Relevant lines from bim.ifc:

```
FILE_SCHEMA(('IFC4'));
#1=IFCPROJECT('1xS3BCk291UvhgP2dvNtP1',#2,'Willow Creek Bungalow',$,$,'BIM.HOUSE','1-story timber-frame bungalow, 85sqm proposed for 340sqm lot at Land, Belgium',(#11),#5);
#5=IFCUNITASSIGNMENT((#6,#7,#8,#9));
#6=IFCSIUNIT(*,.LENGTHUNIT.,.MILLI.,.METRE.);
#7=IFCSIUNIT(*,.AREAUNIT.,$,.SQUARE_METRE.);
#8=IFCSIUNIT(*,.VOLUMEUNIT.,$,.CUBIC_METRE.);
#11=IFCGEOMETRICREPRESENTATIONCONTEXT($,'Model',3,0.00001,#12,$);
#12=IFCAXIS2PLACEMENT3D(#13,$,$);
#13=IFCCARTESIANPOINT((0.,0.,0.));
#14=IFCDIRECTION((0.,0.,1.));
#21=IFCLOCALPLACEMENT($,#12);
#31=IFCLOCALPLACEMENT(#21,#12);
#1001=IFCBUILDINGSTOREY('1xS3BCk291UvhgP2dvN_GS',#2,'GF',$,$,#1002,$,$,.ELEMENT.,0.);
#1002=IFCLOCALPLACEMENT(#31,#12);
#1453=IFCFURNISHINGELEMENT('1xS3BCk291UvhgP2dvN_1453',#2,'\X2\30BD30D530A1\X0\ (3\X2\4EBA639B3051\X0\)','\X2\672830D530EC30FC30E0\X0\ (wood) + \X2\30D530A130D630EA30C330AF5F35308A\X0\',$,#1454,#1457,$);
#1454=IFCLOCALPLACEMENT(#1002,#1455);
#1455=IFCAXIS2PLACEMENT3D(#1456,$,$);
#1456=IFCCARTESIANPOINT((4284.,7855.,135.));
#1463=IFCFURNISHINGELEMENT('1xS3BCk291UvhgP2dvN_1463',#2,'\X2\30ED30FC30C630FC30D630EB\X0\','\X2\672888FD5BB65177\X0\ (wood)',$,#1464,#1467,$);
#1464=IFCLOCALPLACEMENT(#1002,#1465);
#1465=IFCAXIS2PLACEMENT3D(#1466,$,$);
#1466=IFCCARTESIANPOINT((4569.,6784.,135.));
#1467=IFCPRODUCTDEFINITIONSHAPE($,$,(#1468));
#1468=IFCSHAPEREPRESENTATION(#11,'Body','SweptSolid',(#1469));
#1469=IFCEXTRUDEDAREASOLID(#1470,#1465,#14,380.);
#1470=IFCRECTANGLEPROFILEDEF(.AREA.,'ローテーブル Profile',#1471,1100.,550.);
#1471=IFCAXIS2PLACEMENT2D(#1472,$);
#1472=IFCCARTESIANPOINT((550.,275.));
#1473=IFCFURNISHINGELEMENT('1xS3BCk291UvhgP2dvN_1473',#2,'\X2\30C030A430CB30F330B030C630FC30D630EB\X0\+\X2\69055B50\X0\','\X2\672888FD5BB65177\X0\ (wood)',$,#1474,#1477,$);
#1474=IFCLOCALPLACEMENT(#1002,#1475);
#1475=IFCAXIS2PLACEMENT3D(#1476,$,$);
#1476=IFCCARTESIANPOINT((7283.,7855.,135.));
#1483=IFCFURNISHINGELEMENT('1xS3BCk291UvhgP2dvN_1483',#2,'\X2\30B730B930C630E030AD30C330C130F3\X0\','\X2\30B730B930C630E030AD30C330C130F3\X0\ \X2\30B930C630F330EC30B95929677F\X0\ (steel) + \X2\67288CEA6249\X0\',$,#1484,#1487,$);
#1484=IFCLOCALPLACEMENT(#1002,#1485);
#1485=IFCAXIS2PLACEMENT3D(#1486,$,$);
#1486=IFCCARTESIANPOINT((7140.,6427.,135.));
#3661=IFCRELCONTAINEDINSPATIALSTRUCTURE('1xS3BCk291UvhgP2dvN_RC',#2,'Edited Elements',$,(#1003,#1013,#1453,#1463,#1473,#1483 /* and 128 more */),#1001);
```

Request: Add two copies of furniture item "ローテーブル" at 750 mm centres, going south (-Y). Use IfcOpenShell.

```python
import numpy as np
import ifcopenshell
import ifcopenshell.api.geometry
import ifcopenshell.api.root
import ifcopenshell.util.element
import ifcopenshell.util.placement
import ifcopenshell.util.unit

model = ifcopenshell.open("bim.ifc")
unit_scale = ifcopenshell.util.unit.calculate_unit_scale(model)


def reuse_history(source, copy):
    """copy_class also copies each property set's owner history, people and application; keep the originals."""
    for rel in copy.IsDefinedBy:
        if rel.is_a("IfcRelDefinesByProperties") and (history := rel.RelatingPropertyDefinition.OwnerHistory):
            rel.RelatingPropertyDefinition.OwnerHistory = source.OwnerHistory
            ifcopenshell.util.element.remove_deep2(model, history)


source = model.by_guid("1xS3BCk291UvhgP2dvN_1463")
base = ifcopenshell.util.placement.get_local_placement(source.ObjectPlacement)
step = np.array([0.0, -1.0, 0.0]) * 0.75 / unit_scale

for i in range(1, 3):
    copy = ifcopenshell.api.root.copy_class(model, product=source)
    copy.Representation = ifcopenshell.util.element.copy_deep(
        model, source.Representation, exclude=["IfcGeometricRepresentationContext", "IfcRepresentationMap"]
    )
    reuse_history(source, copy)
    matrix = base.copy()
    matrix[:3, 3] += i * step
    print("added at", matrix[:3, 3].round(3) + 0.0)
    ifcopenshell.api.geometry.edit_object_placement(model, product=copy, matrix=matrix, is_si=False)

model.write("bim_edited.ifc")
```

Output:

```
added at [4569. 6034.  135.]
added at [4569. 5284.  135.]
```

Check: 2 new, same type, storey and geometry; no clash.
